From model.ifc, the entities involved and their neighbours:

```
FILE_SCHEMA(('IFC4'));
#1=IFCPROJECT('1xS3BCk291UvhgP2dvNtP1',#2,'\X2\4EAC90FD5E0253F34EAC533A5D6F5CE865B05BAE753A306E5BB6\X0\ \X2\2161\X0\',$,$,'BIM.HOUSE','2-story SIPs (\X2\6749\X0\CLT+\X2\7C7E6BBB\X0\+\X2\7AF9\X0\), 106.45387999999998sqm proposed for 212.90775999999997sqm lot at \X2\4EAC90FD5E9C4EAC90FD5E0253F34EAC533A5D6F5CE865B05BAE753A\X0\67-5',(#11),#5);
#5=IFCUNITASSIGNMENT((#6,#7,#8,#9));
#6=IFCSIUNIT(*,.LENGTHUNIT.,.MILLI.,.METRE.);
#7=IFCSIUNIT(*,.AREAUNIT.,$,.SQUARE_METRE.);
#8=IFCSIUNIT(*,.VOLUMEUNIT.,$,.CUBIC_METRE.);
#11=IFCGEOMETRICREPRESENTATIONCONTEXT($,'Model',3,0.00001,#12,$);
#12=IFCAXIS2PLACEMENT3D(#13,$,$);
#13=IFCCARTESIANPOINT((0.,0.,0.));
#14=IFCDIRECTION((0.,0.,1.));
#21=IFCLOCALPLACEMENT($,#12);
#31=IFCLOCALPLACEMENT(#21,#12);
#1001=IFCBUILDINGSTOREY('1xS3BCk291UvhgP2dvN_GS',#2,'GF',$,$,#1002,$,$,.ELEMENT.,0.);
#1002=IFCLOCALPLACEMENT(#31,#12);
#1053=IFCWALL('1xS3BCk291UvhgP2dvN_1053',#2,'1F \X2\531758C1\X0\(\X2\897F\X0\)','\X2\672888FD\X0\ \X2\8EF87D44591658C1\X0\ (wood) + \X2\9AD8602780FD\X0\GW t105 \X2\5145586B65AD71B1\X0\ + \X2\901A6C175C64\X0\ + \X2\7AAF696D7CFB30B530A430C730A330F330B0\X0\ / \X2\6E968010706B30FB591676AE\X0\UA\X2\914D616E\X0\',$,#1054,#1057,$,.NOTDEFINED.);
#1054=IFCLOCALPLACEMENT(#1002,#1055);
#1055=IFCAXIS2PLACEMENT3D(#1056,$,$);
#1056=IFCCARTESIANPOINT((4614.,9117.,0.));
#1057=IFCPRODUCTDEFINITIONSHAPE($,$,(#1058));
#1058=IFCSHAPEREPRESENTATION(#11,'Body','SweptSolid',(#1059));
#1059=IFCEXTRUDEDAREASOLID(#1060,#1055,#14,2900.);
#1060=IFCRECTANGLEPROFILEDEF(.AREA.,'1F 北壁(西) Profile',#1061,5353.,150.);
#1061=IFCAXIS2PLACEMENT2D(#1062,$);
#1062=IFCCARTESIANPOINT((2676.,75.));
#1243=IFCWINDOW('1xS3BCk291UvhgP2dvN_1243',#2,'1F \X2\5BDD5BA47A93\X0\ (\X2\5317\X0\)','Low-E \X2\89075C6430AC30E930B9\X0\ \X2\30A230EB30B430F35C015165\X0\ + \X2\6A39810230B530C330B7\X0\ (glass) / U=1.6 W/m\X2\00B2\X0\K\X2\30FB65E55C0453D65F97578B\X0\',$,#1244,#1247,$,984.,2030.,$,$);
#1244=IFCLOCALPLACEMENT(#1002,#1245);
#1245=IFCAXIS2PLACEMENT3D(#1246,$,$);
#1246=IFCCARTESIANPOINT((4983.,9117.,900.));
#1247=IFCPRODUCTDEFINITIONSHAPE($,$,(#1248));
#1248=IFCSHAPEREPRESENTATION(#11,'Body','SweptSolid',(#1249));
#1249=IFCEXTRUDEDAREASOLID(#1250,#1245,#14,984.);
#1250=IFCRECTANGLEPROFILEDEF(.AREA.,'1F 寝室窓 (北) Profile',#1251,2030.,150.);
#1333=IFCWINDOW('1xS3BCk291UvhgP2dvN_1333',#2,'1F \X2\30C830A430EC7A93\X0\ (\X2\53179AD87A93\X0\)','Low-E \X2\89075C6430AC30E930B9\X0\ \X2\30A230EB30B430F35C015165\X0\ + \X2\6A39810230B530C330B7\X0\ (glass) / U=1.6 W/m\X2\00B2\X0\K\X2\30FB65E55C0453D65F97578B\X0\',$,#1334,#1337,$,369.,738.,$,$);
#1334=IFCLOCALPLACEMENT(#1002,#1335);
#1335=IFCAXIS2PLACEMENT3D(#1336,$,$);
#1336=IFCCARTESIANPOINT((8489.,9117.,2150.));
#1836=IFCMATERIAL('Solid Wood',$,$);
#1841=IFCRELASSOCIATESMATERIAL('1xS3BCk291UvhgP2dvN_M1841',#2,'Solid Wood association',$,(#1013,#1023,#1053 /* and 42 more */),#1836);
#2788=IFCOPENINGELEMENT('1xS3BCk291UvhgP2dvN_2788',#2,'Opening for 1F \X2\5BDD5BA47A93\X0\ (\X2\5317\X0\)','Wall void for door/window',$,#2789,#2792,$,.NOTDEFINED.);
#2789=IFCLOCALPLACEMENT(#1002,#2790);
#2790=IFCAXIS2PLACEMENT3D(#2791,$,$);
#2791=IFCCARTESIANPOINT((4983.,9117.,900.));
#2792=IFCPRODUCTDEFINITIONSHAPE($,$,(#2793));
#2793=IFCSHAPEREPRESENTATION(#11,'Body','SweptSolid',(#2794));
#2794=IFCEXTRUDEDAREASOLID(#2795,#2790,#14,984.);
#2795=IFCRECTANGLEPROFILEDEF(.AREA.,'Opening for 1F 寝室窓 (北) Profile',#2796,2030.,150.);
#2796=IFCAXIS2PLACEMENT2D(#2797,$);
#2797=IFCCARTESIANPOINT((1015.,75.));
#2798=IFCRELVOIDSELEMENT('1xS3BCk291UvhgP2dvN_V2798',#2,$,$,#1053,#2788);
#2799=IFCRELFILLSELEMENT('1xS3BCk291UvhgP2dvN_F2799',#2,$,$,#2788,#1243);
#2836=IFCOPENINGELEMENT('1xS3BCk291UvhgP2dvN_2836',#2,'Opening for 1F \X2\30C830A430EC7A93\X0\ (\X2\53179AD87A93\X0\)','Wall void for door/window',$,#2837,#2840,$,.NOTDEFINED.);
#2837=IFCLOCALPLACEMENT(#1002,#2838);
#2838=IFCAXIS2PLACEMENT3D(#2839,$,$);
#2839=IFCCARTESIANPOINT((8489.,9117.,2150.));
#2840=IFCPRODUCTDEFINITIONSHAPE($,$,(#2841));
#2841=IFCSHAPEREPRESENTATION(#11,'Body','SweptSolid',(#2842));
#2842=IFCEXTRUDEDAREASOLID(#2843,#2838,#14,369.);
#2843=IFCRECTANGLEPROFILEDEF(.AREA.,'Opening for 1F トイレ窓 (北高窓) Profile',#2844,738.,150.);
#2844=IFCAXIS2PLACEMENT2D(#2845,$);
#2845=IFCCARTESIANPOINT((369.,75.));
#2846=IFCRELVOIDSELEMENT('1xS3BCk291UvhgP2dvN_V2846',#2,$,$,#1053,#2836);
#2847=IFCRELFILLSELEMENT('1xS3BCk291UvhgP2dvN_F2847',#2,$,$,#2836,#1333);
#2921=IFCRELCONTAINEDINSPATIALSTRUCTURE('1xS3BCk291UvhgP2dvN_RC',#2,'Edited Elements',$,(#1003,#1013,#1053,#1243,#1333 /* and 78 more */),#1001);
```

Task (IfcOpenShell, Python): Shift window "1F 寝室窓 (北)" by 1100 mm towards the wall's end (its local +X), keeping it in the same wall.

```python
import ifcopenshell
import ifcopenshell.api.geometry
import ifcopenshell.util.placement
import ifcopenshell.util.unit

model = ifcopenshell.open("model.ifc")
unit_scale = ifcopenshell.util.unit.calculate_unit_scale(model)

window = model.by_guid("1xS3BCk291UvhgP2dvN_1243")
opening = window.FillsVoids[0].RelatingOpeningElement
wall = opening.VoidsElements[0].RelatingBuildingElement

wall_matrix = ifcopenshell.util.placement.get_local_placement(wall.ObjectPlacement)
shift = wall_matrix[:3, 0] * 1.1 / unit_scale
before = ifcopenshell.util.placement.get_local_placement(window.ObjectPlacement)[:3, 3].copy()

# The window is not placed relative to its opening, so move both.
for product in (opening, window):
    matrix = ifcopenshell.util.placement.get_local_placement(product.ObjectPlacement)
    matrix[:3, 3] += shift
    ifcopenshell.api.geometry.edit_object_placement(model, product=product, matrix=matrix, is_si=False)

after = ifcopenshell.util.placement.get_local_placement(window.ObjectPlacement)[:3, 3]
print("window moved by", (after - before).round(3) + 0.0)

model.write("model_updated.ifc")
```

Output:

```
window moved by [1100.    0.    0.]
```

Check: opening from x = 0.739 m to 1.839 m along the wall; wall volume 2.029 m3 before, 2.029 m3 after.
